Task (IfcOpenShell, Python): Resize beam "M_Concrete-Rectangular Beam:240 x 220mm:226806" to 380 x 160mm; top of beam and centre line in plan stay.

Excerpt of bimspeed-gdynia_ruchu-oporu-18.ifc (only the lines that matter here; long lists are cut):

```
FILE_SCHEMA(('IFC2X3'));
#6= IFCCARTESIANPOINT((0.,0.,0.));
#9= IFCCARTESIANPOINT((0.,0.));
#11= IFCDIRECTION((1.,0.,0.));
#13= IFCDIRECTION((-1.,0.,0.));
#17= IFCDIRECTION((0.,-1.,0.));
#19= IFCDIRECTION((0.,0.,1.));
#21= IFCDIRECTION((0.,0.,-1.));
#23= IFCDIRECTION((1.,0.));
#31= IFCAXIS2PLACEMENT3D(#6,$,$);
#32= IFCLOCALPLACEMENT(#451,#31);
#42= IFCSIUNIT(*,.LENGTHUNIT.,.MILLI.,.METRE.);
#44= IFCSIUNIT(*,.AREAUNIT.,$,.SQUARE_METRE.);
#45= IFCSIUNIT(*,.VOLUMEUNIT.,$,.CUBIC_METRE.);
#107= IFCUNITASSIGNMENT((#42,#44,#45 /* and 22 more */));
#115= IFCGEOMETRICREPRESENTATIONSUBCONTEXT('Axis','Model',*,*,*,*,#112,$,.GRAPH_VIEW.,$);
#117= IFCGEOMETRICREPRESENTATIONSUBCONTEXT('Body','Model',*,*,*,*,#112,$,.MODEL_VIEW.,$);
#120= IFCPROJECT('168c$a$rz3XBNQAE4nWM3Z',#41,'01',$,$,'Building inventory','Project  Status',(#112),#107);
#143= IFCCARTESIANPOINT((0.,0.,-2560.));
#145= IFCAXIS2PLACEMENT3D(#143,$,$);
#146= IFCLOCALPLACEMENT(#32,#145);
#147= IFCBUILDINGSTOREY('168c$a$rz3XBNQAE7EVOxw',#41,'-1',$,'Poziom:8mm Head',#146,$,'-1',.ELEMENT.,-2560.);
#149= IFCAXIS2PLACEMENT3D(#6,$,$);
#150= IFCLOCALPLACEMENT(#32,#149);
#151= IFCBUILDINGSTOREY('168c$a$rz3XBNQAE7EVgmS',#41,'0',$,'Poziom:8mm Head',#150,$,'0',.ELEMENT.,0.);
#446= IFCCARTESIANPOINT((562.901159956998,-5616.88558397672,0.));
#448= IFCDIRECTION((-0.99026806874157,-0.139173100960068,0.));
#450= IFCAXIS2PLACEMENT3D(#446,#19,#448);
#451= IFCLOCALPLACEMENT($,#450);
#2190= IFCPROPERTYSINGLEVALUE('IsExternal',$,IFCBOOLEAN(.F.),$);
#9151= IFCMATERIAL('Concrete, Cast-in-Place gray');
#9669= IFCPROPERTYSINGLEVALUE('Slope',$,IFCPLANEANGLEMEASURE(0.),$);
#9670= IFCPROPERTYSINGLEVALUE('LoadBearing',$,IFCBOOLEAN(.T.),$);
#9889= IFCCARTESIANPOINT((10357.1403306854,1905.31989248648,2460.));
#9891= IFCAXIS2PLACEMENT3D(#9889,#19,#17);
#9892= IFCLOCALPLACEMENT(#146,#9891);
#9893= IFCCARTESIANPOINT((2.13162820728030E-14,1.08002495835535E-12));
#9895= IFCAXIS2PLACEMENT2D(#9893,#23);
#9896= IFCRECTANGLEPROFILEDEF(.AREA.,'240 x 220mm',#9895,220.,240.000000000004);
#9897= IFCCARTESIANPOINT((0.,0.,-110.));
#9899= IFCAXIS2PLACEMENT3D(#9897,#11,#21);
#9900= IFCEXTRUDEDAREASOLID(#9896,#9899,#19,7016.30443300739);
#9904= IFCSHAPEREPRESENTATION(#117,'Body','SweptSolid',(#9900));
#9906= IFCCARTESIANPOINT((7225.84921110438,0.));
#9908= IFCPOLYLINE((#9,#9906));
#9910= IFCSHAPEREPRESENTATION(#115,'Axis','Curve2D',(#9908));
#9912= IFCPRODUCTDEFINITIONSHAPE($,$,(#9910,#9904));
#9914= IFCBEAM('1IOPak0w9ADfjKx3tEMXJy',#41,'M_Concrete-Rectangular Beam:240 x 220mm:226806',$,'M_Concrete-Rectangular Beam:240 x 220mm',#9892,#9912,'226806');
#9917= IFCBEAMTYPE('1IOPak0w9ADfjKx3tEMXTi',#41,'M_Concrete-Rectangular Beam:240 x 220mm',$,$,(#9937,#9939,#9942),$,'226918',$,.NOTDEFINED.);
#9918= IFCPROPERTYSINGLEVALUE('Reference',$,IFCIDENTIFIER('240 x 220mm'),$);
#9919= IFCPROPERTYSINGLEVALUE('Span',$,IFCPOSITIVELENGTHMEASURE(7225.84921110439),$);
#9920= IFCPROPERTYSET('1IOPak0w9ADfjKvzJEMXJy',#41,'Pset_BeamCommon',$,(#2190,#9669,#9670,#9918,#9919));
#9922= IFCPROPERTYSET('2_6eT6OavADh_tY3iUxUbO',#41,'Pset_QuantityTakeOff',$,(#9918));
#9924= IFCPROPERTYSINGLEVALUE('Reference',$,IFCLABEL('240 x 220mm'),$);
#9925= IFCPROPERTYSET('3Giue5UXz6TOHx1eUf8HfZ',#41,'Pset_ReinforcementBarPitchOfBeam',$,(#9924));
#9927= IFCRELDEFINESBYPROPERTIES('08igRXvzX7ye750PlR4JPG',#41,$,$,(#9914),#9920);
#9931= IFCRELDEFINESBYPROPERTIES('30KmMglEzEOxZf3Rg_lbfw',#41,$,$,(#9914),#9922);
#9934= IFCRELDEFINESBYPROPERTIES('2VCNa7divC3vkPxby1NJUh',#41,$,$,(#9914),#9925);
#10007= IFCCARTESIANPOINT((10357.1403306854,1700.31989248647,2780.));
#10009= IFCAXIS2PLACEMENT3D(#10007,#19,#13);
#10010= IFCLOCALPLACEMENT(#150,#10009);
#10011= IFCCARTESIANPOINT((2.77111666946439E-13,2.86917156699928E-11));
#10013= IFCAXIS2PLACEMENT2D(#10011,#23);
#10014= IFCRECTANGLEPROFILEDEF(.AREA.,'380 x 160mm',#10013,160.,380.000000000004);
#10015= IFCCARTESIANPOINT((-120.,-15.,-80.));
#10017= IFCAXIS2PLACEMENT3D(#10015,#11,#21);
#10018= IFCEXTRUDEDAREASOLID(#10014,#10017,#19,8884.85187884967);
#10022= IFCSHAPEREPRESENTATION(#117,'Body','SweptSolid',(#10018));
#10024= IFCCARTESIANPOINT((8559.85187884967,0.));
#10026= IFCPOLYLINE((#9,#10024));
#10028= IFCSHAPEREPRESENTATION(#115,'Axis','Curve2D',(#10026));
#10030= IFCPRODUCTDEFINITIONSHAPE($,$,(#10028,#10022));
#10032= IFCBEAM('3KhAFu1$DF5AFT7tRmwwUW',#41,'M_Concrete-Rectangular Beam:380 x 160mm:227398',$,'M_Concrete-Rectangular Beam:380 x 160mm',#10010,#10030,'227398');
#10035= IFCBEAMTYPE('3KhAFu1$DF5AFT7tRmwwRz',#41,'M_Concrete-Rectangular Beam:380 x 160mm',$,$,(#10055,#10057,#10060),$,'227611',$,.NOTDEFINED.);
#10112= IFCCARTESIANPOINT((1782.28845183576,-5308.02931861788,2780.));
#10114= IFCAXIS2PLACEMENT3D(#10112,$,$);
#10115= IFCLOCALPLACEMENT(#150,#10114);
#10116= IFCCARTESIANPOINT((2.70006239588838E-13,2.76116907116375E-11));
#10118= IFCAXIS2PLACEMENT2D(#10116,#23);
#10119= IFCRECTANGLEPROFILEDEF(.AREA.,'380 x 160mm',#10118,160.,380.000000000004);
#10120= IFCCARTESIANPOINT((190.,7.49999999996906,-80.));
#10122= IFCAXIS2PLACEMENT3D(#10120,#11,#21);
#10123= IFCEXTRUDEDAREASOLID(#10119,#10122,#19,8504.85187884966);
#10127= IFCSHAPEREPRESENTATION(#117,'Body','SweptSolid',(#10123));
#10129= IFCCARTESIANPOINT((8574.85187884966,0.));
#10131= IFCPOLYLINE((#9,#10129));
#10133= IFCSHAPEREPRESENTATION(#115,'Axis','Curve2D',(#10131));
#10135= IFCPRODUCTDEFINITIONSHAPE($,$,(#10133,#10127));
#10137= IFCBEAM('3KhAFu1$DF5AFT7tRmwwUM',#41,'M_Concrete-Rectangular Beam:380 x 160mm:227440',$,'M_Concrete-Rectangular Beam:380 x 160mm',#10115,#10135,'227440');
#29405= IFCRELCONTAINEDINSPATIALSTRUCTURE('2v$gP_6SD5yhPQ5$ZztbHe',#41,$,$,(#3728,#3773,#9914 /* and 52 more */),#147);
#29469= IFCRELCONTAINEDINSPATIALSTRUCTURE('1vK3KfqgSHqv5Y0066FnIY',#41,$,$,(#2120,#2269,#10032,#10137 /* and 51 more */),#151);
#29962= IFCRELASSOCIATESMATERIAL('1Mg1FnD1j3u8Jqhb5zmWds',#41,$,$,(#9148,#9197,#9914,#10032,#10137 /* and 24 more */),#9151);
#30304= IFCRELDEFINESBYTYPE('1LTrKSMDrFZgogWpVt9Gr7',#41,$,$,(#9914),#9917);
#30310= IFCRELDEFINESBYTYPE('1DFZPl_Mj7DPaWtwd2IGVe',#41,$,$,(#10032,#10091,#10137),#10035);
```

```python
import ifcopenshell
import ifcopenshell.api.pset
import ifcopenshell.api.type
import ifcopenshell.util.element
import ifcopenshell.util.representation

model = ifcopenshell.open("bimspeed-gdynia_ruchu-oporu-18.ifc")

member = model.by_guid("1IOPak0w9ADfjKx3tEMXJy")
source = next(p for p in model.by_type("IfcRectangleProfileDef") if p.ProfileName == "380 x 160mm")

body = ifcopenshell.util.representation.get_representation(member, "Model", "Body")
solid = body.Items[0]
old_profile = solid.SweptArea

# Copy the section's sizes but keep this member's own profile position.
profile = ifcopenshell.util.element.copy(model, source)
# Profiles are centred, so shift by half the change in depth to hold the top.
shift = (old_profile.XDim - profile.XDim) / 2
x, y = old_profile.Position.Location.Coordinates
up = (-1.0, 0.0)  # upwards, in the solid's own plane
location = model.createIfcCartesianPoint((x + up[0] * shift, y + up[1] * shift))
profile.Position = model.createIfcAxis2Placement2D(location, old_profile.Position.RefDirection)
solid.SweptArea = profile
if not model.get_total_inverses(old_profile):
    ifcopenshell.util.element.remove_deep2(model, old_profile)

new_type = model.by_guid("3KhAFu1$DF5AFT7tRmwwRz")
ifcopenshell.api.type.assign_type(
    model, related_objects=[member], relating_type=new_type, should_map_representations=False
)
member.Name = member.Name.replace("240 x 220mm", "380 x 160mm")
member.ObjectType = "M_Concrete-Rectangular Beam:380 x 160mm"
pset = model.by_id(ifcopenshell.util.element.get_pset(member, "Pset_BeamCommon", should_inherit=False)["id"])
ifcopenshell.api.pset.edit_pset(model, pset=pset, properties={"Reference": "380 x 160mm"})
pset = model.by_id(ifcopenshell.util.element.get_pset(member, "Pset_QuantityTakeOff", should_inherit=False)["id"])
ifcopenshell.api.pset.edit_pset(model, pset=pset, properties={"Reference": "380 x 160mm"})
pset = model.by_id(ifcopenshell.util.element.get_pset(member, "Pset_ReinforcementBarPitchOfBeam", should_inherit=False)["id"])
ifcopenshell.api.pset.edit_pset(model, pset=pset, properties={"Reference": "380 x 160mm"})

print(solid.SweptArea)

model.write("bimspeed-gdynia_ruchu-oporu-18-out.ifc")
```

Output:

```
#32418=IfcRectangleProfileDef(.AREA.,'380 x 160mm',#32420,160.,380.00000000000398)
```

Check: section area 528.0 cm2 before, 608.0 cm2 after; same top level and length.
